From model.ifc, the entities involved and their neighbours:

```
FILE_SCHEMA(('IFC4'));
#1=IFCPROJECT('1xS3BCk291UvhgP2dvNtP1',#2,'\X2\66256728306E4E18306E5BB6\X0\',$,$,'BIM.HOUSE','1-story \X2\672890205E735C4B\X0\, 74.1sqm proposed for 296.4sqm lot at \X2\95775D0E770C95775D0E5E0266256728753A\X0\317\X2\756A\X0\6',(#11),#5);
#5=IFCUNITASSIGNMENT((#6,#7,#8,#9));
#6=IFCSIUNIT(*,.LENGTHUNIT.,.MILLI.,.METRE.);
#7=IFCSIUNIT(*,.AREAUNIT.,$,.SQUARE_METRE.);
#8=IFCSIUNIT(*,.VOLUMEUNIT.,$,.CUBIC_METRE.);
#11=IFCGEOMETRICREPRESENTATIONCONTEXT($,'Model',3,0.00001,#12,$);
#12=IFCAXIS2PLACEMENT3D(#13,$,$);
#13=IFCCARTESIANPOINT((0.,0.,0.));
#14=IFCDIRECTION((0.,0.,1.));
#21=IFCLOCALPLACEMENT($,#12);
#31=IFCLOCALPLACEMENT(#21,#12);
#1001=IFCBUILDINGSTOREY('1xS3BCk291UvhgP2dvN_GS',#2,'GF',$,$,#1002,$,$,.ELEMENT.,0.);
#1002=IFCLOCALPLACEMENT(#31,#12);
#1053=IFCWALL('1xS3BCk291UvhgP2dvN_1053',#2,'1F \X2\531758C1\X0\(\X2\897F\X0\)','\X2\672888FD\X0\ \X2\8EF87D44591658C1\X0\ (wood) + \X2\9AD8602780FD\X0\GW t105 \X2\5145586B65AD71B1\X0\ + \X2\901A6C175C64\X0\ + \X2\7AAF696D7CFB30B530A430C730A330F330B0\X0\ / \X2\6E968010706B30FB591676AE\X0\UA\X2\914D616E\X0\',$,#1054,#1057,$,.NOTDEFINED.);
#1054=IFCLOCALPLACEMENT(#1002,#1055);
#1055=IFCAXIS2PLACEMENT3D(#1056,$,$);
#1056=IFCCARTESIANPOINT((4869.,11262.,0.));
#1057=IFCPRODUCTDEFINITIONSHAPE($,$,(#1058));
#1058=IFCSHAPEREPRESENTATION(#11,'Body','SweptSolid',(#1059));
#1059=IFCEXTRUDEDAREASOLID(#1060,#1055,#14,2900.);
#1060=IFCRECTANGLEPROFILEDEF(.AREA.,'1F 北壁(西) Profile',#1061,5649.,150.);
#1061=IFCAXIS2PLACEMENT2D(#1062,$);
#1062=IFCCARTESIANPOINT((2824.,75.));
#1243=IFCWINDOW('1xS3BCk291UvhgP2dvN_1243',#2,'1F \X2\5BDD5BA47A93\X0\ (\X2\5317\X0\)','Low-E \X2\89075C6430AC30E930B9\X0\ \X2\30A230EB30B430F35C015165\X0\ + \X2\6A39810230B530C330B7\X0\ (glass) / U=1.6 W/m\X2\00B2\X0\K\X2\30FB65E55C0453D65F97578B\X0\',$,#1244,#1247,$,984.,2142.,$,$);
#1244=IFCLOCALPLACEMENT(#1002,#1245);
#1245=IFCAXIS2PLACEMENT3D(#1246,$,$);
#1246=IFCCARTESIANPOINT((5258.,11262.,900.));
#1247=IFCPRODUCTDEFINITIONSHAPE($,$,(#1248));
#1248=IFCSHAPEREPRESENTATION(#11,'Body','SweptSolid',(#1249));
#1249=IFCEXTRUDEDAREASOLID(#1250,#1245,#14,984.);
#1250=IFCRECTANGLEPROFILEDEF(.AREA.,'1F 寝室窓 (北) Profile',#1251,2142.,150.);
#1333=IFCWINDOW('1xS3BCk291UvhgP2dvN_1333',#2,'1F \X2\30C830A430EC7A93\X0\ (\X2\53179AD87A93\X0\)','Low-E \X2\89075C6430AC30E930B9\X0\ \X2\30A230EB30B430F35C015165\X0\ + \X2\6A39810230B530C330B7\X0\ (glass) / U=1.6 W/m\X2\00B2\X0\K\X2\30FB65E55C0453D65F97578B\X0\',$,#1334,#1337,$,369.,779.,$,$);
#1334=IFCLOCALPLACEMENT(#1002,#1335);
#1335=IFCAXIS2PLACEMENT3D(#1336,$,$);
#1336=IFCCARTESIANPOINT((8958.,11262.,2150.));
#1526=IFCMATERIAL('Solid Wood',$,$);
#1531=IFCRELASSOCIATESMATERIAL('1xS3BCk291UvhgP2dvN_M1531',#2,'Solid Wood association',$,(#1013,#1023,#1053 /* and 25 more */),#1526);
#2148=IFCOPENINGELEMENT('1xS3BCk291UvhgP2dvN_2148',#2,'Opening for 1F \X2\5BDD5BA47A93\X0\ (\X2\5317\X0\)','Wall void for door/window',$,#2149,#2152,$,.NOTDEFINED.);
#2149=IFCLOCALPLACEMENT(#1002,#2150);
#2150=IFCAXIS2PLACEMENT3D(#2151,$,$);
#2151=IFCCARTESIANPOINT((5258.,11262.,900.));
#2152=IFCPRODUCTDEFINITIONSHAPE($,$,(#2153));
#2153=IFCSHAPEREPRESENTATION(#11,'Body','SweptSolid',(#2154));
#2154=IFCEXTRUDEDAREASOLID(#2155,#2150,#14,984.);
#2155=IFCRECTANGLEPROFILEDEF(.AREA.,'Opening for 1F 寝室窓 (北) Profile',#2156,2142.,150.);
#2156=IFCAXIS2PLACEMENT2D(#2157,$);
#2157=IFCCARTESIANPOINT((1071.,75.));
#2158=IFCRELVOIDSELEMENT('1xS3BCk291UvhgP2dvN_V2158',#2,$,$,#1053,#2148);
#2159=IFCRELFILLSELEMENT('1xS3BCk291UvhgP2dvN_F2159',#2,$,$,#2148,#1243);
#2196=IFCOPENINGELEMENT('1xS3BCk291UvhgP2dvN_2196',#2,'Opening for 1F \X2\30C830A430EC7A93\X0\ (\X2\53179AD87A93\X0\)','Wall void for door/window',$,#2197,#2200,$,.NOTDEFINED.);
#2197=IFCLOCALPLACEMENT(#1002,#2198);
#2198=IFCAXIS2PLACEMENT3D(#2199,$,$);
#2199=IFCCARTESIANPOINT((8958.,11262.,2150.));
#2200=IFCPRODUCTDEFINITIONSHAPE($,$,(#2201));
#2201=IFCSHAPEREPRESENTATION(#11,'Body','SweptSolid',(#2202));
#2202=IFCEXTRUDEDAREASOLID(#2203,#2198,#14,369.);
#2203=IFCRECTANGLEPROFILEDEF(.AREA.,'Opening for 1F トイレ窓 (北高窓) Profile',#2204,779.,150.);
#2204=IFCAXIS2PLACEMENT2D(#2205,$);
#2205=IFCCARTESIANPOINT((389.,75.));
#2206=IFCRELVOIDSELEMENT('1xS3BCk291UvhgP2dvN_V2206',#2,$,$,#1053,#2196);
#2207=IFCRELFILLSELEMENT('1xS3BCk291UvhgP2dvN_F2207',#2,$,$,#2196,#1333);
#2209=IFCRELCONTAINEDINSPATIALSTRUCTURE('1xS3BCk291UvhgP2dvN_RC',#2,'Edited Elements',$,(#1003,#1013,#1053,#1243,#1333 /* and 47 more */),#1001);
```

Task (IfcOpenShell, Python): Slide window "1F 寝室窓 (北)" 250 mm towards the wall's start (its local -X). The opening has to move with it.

```python
import ifcopenshell
import ifcopenshell.api.geometry
import ifcopenshell.util.placement
import ifcopenshell.util.unit

model = ifcopenshell.open("model.ifc")
unit_scale = ifcopenshell.util.unit.calculate_unit_scale(model)

window = model.by_guid("1xS3BCk291UvhgP2dvN_1243")
opening = window.FillsVoids[0].RelatingOpeningElement
wall = opening.VoidsElements[0].RelatingBuildingElement

wall_matrix = ifcopenshell.util.placement.get_local_placement(wall.ObjectPlacement)
shift = wall_matrix[:3, 0] * -0.25 / unit_scale
before = ifcopenshell.util.placement.get_local_placement(window.ObjectPlacement)[:3, 3].copy()

# The window is not placed relative to its opening, so move both.
for product in (opening, window):
    matrix = ifcopenshell.util.placement.get_local_placement(product.ObjectPlacement)
    matrix[:3, 3] += shift
    ifcopenshell.api.geometry.edit_object_placement(model, product=product, matrix=matrix, is_si=False)

after = ifcopenshell.util.placement.get_local_placement(window.ObjectPlacement)[:3, 3]
print("window moved by", (after - before).round(3) + 0.0)

model.write("model_updated.ifc")
```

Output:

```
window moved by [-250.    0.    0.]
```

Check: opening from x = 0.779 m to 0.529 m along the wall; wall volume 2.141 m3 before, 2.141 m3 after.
